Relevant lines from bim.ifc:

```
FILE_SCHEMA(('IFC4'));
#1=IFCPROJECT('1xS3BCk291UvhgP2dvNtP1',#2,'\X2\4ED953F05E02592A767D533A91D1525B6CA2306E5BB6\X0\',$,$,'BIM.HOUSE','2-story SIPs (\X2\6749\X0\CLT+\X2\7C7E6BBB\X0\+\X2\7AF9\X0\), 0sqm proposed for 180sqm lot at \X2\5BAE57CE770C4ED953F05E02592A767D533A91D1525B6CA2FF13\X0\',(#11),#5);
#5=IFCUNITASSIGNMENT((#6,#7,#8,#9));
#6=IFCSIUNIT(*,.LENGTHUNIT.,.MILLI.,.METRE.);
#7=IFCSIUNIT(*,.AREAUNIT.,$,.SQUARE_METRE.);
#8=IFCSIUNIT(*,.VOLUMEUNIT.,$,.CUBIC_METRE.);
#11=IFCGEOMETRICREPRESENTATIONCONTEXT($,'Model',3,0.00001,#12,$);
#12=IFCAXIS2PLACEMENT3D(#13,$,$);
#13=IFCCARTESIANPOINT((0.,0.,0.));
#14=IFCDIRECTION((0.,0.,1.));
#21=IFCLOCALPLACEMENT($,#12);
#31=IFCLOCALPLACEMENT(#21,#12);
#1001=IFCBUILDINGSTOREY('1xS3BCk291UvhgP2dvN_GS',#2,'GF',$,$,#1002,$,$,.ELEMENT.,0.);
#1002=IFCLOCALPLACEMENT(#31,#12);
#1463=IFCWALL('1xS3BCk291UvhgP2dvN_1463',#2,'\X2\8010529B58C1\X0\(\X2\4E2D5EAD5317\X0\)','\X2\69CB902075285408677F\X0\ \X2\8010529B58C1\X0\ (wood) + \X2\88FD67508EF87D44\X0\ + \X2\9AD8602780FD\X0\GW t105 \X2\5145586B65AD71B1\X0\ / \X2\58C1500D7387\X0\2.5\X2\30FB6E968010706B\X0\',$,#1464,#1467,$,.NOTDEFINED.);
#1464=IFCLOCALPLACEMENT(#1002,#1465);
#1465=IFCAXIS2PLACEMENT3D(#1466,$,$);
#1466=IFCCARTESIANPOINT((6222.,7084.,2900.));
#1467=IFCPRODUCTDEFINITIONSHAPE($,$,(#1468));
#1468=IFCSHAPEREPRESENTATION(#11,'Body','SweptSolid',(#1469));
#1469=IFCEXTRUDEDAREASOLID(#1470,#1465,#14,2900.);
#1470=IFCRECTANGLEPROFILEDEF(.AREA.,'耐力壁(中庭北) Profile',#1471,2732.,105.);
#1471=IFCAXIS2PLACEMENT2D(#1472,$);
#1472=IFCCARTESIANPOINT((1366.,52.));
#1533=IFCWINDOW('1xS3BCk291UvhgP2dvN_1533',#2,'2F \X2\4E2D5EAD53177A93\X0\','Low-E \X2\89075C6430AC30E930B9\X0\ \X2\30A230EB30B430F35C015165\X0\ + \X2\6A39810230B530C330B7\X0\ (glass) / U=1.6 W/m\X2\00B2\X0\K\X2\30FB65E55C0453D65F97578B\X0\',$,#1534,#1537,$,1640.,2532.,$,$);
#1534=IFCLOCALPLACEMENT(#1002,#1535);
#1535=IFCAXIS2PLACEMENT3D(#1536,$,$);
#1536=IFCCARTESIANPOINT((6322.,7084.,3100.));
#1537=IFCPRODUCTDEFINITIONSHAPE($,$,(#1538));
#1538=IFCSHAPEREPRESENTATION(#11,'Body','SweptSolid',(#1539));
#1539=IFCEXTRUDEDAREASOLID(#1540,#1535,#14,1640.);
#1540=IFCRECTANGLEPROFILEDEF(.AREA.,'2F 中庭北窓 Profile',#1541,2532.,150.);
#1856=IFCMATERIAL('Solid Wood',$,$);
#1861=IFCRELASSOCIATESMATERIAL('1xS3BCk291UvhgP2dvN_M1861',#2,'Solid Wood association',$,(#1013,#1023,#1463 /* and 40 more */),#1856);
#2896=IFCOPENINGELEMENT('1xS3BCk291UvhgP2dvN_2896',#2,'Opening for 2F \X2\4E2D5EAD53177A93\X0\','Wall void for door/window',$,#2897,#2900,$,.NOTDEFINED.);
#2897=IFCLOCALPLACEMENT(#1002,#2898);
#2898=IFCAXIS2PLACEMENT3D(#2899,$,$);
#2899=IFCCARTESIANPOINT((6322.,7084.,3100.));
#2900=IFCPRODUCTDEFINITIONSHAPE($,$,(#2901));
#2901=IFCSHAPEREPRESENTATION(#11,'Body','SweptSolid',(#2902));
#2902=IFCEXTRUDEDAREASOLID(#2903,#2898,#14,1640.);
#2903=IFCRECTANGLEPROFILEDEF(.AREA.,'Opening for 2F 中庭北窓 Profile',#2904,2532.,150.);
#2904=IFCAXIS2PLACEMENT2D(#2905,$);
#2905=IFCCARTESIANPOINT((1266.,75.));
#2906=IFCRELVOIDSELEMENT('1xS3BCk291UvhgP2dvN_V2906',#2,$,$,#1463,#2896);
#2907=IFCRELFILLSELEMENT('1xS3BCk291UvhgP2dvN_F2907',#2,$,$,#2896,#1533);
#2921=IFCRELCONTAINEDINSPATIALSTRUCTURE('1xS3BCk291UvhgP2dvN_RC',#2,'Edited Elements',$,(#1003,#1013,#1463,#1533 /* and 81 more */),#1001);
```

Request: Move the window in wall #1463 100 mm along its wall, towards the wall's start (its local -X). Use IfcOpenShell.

```python
import ifcopenshell
import ifcopenshell.api.geometry
import ifcopenshell.util.placement
import ifcopenshell.util.unit

model = ifcopenshell.open("bim.ifc")
unit_scale = ifcopenshell.util.unit.calculate_unit_scale(model)

window = model.by_guid("1xS3BCk291UvhgP2dvN_1533")
opening = window.FillsVoids[0].RelatingOpeningElement
wall = opening.VoidsElements[0].RelatingBuildingElement

wall_matrix = ifcopenshell.util.placement.get_local_placement(wall.ObjectPlacement)
shift = wall_matrix[:3, 0] * -0.1 / unit_scale
before = ifcopenshell.util.placement.get_local_placement(window.ObjectPlacement)[:3, 3].copy()

# The window is not placed relative to its opening, so move both.
for product in (opening, window):
    matrix = ifcopenshell.util.placement.get_local_placement(product.ObjectPlacement)
    matrix[:3, 3] += shift
    ifcopenshell.api.geometry.edit_object_placement(model, product=product, matrix=matrix, is_si=False)

after = ifcopenshell.util.placement.get_local_placement(window.ObjectPlacement)[:3, 3]
print("window moved by", (after - before).round(3) + 0.0)

model.write("bim_v2.ifc")
```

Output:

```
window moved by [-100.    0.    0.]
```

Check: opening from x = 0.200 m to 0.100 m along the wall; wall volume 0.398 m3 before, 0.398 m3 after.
